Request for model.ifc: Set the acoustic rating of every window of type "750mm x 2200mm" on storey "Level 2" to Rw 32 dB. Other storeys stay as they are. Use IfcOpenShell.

First a look at what the model holds.

```python
import ifcopenshell
import ifcopenshell.util.element

model = ifcopenshell.open("model.ifc")
print(model.schema)
storey = next(s for s in model.by_type("IfcBuildingStorey") if s.Name == "Level 2")
windows = [e for e in ifcopenshell.util.element.get_decomposition(storey) if e.is_a("IfcWindow")]
seen = {}
for e in windows:
    element_type = ifcopenshell.util.element.get_type(e)
    key = (element_type.Name if element_type != e and element_type else None, ifcopenshell.util.element.get_pset(e, "Pset_WindowCommon", "AcousticRating"))
    seen[key] = seen.get(key, 0) + 1
for (name, value), count in sorted(seen.items(), key=str):
    print(count, "x", name, "|", value)
```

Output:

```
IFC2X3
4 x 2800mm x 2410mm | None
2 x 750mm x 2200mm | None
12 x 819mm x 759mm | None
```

```python
import ifcopenshell
import ifcopenshell.api.pset
import ifcopenshell.util.element

model = ifcopenshell.open("model.ifc")

storey = next(s for s in model.by_type("IfcBuildingStorey") if s.Name == "Level 2")
windows = [e for e in ifcopenshell.util.element.get_decomposition(storey) if e.is_a("IfcWindow")]

count = 0
for e in windows:
    element_type = ifcopenshell.util.element.get_type(e)
    if element_type in (None, e) or element_type.Name != "750mm x 2200mm":
        continue
    # add_pset returns the element's existing set when there is one.
    pset = ifcopenshell.api.pset.add_pset(model, product=e, name="Pset_WindowCommon")
    ifcopenshell.api.pset.edit_pset(model, pset=pset, properties={"AcousticRating": "Rw 32 dB"})
    count += 1

print(count, "windows updated")

model.write("model_updated.ifc")
```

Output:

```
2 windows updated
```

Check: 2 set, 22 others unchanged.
